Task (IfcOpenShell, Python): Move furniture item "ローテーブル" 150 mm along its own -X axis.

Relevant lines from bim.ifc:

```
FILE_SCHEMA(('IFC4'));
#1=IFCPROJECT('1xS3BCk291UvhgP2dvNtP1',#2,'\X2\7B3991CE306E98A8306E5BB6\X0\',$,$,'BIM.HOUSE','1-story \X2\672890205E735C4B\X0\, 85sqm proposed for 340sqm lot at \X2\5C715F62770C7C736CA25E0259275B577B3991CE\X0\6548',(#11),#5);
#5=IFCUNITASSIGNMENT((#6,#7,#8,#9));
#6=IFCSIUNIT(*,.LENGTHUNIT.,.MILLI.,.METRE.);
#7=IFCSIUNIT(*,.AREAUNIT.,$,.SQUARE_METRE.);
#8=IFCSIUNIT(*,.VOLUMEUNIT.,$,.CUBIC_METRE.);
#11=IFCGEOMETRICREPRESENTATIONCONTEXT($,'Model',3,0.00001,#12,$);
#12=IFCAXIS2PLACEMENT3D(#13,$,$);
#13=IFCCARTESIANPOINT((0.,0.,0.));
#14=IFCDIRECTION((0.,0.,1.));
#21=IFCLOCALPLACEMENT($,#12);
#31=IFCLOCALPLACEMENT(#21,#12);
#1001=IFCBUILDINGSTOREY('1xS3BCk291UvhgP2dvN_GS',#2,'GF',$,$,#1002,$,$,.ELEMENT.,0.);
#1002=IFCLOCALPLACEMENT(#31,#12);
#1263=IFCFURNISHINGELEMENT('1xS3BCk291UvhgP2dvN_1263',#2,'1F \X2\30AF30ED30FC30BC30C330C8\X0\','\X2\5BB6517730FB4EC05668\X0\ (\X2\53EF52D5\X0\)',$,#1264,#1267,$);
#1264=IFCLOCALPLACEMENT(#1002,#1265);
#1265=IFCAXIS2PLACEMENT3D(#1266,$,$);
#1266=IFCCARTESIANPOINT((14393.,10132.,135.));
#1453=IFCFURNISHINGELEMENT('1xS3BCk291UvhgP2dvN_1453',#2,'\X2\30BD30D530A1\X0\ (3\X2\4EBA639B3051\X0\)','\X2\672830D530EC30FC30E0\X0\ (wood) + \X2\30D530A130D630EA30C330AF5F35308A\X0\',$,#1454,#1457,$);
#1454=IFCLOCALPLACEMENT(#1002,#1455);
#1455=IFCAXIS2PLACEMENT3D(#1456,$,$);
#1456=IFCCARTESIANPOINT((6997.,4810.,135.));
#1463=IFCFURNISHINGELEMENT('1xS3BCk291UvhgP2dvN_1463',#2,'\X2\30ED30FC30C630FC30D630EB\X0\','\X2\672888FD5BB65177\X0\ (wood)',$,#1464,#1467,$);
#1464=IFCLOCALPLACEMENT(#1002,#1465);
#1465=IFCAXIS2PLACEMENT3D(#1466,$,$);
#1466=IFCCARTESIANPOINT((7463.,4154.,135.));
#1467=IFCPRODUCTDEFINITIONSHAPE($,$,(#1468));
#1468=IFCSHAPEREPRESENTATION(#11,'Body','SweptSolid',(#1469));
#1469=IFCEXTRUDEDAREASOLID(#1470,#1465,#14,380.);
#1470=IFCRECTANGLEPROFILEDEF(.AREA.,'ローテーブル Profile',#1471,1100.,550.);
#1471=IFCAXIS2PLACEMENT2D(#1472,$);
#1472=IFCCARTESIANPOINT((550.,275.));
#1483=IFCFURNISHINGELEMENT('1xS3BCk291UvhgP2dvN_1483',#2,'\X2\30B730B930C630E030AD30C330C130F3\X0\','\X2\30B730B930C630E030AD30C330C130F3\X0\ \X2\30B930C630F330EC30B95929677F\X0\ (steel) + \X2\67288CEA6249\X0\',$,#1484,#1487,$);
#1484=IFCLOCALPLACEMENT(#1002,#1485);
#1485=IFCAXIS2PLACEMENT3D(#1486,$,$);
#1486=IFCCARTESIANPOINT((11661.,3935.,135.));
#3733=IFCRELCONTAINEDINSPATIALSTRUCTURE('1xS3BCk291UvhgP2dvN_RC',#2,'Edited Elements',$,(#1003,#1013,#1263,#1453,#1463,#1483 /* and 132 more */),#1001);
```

```python
import ifcopenshell
import ifcopenshell.api.geometry
import ifcopenshell.util.placement

model = ifcopenshell.open("bim.ifc")

item = model.by_id(1463)
matrix = ifcopenshell.util.placement.get_local_placement(item.ObjectPlacement)
matrix[:3, 3] -= matrix[:3, 0] * 150.0
ifcopenshell.api.geometry.edit_object_placement(model, product=item, matrix=matrix, is_si=False)

print(ifcopenshell.util.placement.get_local_placement(item.ObjectPlacement).round(3) + 0.0)

model.write("bim-out.ifc")
```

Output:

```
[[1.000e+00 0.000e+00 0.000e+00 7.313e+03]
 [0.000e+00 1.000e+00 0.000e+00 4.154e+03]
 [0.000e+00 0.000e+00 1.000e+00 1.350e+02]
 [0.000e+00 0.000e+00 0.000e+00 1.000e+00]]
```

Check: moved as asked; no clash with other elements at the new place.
